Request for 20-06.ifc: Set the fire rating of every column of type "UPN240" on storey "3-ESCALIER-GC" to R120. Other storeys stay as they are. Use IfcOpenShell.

First a look at what the model holds.

```python
import ifcopenshell
import ifcopenshell.util.element

model = ifcopenshell.open("20-06.ifc")
print(model.schema)
storey = next(s for s in model.by_type("IfcBuildingStorey") if s.Name == "3-ESCALIER-GC")
columns = [e for e in ifcopenshell.util.element.get_decomposition(storey) if e.is_a("IfcColumn")]
seen = {}
for e in columns:
    element_type = ifcopenshell.util.element.get_type(e)
    key = (element_type.Name if element_type != e and element_type else None, ifcopenshell.util.element.get_pset(e, "Pset_ColumnCommon", "FireRating"))
    seen[key] = seen.get(key, 0) + 1
for (name, value), count in sorted(seen.items(), key=str):
    print(count, "x", name, "|", value)
```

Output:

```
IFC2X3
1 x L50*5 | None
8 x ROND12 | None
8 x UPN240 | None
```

```python
import ifcopenshell
import ifcopenshell.api.pset
import ifcopenshell.util.element

model = ifcopenshell.open("20-06.ifc")

storey = next(s for s in model.by_type("IfcBuildingStorey") if s.Name == "3-ESCALIER-GC")
columns = [e for e in ifcopenshell.util.element.get_decomposition(storey) if e.is_a("IfcColumn")]

count = 0
for e in columns:
    element_type = ifcopenshell.util.element.get_type(e)
    if element_type in (None, e) or element_type.Name != "UPN240":
        continue
    # add_pset returns the element's existing set when there is one.
    pset = ifcopenshell.api.pset.add_pset(model, product=e, name="Pset_ColumnCommon")
    ifcopenshell.api.pset.edit_pset(model, pset=pset, properties={"FireRating": "R120"})
    count += 1

print(count, "columns updated")

model.write("20-06_edited.ifc")
```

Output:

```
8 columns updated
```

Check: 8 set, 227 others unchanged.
